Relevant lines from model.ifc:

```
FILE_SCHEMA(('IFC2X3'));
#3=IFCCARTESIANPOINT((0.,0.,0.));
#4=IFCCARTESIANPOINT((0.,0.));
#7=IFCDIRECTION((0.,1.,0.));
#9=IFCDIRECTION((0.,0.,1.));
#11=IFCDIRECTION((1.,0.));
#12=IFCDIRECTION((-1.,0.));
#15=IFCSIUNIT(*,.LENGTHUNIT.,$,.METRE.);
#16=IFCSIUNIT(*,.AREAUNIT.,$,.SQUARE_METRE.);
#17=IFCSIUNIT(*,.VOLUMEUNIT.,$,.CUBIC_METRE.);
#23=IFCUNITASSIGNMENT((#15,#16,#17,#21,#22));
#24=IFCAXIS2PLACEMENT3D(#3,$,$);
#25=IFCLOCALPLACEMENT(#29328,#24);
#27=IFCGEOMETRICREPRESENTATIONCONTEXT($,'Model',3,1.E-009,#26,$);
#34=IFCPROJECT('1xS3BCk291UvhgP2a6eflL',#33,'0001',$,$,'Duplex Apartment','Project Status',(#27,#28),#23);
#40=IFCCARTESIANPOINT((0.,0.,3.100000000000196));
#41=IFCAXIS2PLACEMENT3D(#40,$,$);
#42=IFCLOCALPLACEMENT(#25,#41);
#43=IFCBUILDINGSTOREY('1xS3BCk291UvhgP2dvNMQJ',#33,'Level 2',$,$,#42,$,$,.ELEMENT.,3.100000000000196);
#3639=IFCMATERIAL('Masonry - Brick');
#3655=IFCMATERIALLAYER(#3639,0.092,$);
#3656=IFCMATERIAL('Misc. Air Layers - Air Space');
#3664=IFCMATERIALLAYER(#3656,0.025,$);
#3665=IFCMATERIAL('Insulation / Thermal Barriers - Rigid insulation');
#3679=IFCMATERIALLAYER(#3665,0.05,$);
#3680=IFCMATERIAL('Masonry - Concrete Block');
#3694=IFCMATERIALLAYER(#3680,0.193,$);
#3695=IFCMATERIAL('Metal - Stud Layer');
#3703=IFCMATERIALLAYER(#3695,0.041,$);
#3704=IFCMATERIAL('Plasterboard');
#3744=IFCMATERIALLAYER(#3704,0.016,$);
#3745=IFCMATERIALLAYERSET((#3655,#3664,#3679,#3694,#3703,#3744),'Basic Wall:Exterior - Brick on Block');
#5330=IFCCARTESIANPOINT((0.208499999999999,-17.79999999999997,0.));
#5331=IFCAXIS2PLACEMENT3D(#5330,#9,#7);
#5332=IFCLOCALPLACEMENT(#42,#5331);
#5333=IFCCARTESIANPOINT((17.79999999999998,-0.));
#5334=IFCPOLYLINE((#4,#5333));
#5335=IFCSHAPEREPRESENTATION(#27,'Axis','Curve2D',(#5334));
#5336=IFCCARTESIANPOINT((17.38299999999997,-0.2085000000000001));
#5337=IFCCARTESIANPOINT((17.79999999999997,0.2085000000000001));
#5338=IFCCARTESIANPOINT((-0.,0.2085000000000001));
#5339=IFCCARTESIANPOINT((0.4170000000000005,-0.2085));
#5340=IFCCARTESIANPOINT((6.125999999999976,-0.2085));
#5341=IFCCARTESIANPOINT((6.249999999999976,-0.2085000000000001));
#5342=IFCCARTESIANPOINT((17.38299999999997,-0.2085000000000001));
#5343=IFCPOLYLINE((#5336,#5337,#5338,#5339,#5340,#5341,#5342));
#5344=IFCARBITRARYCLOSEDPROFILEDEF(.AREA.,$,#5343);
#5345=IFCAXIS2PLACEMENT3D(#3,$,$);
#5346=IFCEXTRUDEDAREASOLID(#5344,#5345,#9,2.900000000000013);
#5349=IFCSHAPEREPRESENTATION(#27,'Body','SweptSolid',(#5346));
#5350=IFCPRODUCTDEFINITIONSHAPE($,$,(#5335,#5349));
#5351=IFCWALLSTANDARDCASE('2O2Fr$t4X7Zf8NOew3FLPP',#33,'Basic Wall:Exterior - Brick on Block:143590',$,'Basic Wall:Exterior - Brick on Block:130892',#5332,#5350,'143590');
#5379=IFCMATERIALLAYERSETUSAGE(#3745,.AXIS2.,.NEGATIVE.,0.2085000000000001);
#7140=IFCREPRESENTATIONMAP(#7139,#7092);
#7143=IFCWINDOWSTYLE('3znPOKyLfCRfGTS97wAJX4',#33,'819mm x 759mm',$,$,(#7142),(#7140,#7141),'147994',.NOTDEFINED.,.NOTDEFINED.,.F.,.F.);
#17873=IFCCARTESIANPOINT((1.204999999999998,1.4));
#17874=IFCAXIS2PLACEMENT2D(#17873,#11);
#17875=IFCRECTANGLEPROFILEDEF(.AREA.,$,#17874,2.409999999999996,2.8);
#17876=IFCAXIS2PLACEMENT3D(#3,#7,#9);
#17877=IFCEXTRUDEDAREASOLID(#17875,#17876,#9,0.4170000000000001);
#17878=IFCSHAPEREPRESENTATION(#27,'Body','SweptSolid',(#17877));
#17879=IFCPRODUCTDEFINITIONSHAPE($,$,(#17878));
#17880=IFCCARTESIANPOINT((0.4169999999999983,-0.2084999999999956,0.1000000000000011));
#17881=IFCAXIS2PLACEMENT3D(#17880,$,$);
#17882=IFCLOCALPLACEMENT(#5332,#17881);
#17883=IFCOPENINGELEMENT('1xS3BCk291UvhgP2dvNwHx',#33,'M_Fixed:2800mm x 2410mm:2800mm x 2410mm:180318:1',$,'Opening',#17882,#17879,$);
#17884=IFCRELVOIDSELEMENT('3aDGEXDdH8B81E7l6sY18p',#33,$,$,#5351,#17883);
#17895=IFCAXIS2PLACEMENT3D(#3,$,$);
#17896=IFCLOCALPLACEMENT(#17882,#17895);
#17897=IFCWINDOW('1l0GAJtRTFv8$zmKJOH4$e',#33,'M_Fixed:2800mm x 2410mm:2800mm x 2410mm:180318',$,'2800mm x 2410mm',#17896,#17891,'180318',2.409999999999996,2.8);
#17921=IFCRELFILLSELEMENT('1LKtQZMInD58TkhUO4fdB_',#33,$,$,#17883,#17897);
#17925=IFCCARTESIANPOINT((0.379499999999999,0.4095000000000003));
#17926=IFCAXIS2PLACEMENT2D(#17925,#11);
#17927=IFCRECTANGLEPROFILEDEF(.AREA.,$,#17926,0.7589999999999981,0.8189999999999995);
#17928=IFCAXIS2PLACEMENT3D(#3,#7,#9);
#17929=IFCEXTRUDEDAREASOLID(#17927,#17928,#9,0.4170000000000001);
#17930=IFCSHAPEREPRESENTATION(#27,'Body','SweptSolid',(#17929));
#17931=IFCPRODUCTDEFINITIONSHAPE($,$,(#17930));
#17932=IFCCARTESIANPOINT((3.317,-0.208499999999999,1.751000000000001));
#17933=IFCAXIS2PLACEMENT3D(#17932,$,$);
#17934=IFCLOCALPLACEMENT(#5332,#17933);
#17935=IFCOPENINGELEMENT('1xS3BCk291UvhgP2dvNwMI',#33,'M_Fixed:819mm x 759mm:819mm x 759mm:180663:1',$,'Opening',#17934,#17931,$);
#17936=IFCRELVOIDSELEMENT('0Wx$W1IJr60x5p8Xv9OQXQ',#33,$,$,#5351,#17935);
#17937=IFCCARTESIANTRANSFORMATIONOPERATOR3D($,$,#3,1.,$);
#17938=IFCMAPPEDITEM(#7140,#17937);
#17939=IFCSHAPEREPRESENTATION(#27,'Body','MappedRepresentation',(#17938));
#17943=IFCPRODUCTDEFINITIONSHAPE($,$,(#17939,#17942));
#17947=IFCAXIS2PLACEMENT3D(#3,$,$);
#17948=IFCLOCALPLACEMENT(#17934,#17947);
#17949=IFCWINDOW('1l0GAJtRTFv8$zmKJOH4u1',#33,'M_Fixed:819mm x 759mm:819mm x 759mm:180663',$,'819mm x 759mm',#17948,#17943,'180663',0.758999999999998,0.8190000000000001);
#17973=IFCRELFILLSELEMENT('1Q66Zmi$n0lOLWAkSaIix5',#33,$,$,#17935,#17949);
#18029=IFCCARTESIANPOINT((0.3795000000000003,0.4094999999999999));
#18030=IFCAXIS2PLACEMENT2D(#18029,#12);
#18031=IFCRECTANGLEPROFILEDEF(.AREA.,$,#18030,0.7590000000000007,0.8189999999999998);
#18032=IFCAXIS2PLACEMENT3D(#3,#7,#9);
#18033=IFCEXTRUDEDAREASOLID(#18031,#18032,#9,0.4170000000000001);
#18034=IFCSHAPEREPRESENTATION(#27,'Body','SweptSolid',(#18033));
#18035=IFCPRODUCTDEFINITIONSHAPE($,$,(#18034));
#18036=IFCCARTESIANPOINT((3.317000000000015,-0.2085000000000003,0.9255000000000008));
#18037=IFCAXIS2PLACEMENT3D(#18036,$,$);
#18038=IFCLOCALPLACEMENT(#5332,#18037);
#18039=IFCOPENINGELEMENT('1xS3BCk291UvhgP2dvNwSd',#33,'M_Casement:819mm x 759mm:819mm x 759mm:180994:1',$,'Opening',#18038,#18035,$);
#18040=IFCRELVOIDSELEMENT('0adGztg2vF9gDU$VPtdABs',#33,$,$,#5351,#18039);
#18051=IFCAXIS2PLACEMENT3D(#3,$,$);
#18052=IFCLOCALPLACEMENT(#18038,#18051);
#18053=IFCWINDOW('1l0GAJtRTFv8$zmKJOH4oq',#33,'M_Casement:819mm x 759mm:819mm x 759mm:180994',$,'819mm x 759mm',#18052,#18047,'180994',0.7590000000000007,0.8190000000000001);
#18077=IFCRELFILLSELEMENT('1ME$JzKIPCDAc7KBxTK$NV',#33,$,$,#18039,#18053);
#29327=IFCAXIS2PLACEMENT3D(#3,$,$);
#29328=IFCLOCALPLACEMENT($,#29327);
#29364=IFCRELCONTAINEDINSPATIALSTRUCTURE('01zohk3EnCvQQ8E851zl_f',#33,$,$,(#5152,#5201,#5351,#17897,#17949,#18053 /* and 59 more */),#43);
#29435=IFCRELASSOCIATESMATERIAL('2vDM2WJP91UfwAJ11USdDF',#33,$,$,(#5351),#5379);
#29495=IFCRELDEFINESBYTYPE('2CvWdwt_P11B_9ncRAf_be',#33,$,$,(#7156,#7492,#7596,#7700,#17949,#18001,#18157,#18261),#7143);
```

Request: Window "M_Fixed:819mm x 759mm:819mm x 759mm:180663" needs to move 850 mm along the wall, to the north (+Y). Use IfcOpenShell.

```python
import ifcopenshell
import ifcopenshell.api.geometry
import ifcopenshell.util.placement
import ifcopenshell.util.unit

model = ifcopenshell.open("model.ifc")
unit_scale = ifcopenshell.util.unit.calculate_unit_scale(model)

window = model.by_guid("1l0GAJtRTFv8$zmKJOH4u1")
opening = window.FillsVoids[0].RelatingOpeningElement
wall = opening.VoidsElements[0].RelatingBuildingElement

wall_matrix = ifcopenshell.util.placement.get_local_placement(wall.ObjectPlacement)
shift = wall_matrix[:3, 0] * 0.85 / unit_scale
before = ifcopenshell.util.placement.get_local_placement(window.ObjectPlacement)[:3, 3].copy()

# The window is placed relative to its opening, so it follows when the opening moves.
matrix = ifcopenshell.util.placement.get_local_placement(opening.ObjectPlacement)
matrix[:3, 3] += shift
ifcopenshell.api.geometry.edit_object_placement(
    model, product=opening, matrix=matrix, is_si=False, should_transform_children=True
)

after = ifcopenshell.util.placement.get_local_placement(window.ObjectPlacement)[:3, 3]
print("window moved by", (after - before).round(3) + 0.0)

model.write("model_updated.ifc")
```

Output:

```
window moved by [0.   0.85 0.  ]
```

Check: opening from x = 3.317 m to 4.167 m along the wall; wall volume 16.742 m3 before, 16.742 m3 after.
